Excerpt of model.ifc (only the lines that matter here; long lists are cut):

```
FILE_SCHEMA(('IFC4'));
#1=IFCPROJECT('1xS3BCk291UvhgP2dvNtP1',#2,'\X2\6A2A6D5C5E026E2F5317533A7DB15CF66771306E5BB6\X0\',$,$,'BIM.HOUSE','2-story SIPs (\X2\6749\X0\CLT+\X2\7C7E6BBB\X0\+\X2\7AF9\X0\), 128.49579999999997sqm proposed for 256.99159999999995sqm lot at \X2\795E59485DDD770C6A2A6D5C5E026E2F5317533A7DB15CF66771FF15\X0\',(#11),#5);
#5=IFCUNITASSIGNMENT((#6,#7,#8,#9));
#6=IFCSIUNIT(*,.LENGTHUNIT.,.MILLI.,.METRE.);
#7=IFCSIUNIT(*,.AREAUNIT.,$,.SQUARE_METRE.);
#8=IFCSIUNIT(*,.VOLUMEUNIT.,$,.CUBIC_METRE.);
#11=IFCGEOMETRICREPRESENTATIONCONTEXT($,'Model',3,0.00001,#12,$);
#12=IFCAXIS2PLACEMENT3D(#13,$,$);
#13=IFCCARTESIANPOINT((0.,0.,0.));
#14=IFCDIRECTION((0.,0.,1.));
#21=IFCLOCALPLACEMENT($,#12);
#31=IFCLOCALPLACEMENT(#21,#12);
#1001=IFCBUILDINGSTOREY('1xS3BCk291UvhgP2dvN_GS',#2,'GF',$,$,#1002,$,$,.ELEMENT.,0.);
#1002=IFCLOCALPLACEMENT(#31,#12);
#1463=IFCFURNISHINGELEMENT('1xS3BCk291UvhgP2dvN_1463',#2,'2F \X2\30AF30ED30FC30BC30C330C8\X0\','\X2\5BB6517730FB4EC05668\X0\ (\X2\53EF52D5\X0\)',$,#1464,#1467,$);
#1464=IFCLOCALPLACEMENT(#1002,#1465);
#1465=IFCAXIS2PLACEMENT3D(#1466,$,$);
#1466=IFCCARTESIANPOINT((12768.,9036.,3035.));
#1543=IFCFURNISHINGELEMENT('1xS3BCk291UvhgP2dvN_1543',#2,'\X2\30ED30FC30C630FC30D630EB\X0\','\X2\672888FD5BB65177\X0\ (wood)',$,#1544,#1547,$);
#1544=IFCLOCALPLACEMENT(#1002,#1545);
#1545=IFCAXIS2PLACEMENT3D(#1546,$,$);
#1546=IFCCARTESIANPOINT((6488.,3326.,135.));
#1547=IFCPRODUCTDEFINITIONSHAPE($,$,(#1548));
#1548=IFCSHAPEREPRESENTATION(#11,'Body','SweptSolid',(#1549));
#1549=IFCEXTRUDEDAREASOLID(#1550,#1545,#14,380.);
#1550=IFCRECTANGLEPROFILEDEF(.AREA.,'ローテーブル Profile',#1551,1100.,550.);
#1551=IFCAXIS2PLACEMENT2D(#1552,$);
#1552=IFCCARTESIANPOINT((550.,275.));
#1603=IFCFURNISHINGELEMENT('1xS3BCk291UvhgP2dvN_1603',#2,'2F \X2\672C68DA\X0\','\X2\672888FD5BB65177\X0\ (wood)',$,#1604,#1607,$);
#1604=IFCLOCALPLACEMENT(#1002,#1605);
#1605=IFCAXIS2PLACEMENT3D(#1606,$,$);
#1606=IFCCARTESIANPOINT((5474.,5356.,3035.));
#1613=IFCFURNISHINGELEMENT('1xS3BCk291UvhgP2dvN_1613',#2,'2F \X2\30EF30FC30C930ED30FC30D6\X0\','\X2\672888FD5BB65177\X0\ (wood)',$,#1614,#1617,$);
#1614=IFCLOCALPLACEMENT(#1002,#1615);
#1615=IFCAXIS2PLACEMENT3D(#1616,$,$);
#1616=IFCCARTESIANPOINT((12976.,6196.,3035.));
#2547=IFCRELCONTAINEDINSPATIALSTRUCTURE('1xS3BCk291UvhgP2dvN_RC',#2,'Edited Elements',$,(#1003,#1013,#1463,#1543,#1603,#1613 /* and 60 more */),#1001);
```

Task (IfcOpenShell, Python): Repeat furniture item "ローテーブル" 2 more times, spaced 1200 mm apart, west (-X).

```python
import numpy as np
import ifcopenshell
import ifcopenshell.api.geometry
import ifcopenshell.api.root
import ifcopenshell.util.element
import ifcopenshell.util.placement

model = ifcopenshell.open("model.ifc")


def reuse_history(source, copy):
    """copy_class also copies each property set's owner history, people and application; keep the originals."""
    for rel in copy.IsDefinedBy:
        if rel.is_a("IfcRelDefinesByProperties") and (history := rel.RelatingPropertyDefinition.OwnerHistory):
            rel.RelatingPropertyDefinition.OwnerHistory = source.OwnerHistory
            ifcopenshell.util.element.remove_deep2(model, history)


source = model.by_id(1543)
base = ifcopenshell.util.placement.get_local_placement(source.ObjectPlacement)
step = np.array([-1.0, 0.0, 0.0]) * 1200.0

for i in range(1, 3):
    copy = ifcopenshell.api.root.copy_class(model, product=source)
    copy.Representation = ifcopenshell.util.element.copy_deep(
        model, source.Representation, exclude=["IfcGeometricRepresentationContext", "IfcRepresentationMap"]
    )
    reuse_history(source, copy)
    matrix = base.copy()
    matrix[:3, 3] += i * step
    print("added at", matrix[:3, 3].round(3) + 0.0)
    ifcopenshell.api.geometry.edit_object_placement(model, product=copy, matrix=matrix, is_si=False)

model.write("model_edited.ifc")
```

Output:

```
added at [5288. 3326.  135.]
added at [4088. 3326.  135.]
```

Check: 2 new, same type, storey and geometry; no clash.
